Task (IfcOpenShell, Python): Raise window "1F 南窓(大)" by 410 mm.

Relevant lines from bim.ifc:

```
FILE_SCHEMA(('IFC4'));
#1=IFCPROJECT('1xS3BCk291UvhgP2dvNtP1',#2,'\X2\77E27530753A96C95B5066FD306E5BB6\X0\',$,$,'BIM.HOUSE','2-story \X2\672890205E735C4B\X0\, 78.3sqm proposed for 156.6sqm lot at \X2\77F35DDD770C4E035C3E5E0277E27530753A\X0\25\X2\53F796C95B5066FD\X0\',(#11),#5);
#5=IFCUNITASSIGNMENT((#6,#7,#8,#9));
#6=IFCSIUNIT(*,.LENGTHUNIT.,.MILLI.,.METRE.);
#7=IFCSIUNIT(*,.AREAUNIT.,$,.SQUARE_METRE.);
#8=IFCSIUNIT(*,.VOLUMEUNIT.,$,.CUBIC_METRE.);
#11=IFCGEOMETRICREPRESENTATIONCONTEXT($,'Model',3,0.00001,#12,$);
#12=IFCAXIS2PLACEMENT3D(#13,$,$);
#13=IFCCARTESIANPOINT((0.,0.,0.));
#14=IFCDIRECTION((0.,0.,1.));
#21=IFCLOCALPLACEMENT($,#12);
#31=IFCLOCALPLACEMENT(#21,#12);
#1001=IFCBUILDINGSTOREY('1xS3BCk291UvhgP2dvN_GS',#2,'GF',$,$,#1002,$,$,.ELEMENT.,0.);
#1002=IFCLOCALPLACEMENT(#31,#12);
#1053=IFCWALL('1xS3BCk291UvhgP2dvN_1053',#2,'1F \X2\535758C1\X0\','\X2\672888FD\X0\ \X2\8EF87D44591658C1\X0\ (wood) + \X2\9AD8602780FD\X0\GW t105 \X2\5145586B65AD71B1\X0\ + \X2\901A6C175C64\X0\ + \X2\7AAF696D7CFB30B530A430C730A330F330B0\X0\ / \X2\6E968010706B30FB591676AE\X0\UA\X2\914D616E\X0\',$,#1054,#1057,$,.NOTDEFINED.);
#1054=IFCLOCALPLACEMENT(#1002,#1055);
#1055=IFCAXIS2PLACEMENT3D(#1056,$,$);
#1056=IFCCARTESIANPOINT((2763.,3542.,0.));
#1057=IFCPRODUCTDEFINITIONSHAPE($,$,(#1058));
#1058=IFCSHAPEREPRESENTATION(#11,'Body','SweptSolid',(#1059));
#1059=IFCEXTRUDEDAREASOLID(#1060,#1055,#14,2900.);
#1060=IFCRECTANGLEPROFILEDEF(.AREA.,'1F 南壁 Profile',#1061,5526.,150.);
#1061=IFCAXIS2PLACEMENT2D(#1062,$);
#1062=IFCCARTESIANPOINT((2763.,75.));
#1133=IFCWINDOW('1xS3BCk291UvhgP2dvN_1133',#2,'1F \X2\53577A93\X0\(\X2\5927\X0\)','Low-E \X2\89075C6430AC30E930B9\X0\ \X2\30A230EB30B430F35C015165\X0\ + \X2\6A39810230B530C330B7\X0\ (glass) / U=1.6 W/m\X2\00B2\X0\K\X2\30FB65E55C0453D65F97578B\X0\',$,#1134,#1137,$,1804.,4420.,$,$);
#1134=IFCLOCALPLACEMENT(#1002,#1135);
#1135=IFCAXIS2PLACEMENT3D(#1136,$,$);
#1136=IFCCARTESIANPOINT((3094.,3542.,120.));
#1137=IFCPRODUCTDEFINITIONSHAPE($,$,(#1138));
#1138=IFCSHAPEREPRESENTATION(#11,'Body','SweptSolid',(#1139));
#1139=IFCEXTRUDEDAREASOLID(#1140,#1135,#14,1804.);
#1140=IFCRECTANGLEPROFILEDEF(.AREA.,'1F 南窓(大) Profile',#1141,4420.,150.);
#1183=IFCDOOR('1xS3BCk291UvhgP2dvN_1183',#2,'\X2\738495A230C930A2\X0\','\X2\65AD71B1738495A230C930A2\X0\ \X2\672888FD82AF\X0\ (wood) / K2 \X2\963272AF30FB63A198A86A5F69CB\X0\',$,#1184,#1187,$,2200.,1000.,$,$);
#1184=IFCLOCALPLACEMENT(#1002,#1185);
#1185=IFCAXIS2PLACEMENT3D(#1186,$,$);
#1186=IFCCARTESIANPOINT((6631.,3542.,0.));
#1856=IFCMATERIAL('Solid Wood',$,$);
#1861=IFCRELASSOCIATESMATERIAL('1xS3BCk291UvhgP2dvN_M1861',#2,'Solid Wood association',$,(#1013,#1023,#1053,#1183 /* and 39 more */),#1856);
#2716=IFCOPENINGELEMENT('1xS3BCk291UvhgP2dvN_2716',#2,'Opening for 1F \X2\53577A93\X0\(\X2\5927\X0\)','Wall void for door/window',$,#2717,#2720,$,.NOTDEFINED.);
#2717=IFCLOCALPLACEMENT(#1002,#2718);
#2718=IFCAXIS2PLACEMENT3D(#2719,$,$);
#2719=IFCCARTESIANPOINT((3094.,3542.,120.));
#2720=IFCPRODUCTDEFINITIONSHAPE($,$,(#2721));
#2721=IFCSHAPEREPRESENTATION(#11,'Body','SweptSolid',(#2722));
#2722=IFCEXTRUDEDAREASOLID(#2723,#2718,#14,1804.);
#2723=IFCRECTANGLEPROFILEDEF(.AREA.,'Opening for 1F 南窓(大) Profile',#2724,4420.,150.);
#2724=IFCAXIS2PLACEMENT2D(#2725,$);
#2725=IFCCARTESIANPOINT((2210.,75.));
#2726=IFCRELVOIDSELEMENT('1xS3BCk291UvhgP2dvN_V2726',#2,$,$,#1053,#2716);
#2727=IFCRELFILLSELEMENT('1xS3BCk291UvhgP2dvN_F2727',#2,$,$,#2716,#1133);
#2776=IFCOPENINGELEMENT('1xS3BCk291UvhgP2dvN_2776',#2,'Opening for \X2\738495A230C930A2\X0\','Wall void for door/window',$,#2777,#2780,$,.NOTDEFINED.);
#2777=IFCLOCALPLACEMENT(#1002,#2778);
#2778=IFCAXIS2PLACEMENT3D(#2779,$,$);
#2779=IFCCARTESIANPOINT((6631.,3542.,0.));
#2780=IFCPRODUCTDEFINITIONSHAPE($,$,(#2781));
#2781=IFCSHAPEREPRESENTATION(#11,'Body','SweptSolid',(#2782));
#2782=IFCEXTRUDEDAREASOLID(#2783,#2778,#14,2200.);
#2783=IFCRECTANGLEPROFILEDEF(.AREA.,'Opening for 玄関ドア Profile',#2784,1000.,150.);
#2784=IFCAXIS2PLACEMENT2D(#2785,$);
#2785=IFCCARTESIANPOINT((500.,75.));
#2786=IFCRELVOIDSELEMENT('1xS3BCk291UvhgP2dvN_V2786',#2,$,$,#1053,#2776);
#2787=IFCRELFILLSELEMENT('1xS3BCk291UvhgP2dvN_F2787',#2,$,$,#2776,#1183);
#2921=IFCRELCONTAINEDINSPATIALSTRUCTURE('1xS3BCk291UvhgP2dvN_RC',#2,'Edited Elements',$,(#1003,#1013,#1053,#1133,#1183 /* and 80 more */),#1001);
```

```python
import numpy as np
import ifcopenshell
import ifcopenshell.api.geometry
import ifcopenshell.util.placement
import ifcopenshell.util.unit

model = ifcopenshell.open("bim.ifc")
unit_scale = ifcopenshell.util.unit.calculate_unit_scale(model)

window = model.by_guid("1xS3BCk291UvhgP2dvN_1133")
opening = window.FillsVoids[0].RelatingOpeningElement
dz = 0.41 / unit_scale

shift = np.array([0.0, 0.0, dz])
# The window is not placed relative to its opening, so move both.
for product in (opening, window):
    matrix = ifcopenshell.util.placement.get_local_placement(product.ObjectPlacement)
    matrix[:3, 3] += shift
    ifcopenshell.api.geometry.edit_object_placement(model, product=product, matrix=matrix, is_si=False)

print(f"moved by {dz * unit_scale:+.3f} m")

model.write("bim_v2.ifc")
```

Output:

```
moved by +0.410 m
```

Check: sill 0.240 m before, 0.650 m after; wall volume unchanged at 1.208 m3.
